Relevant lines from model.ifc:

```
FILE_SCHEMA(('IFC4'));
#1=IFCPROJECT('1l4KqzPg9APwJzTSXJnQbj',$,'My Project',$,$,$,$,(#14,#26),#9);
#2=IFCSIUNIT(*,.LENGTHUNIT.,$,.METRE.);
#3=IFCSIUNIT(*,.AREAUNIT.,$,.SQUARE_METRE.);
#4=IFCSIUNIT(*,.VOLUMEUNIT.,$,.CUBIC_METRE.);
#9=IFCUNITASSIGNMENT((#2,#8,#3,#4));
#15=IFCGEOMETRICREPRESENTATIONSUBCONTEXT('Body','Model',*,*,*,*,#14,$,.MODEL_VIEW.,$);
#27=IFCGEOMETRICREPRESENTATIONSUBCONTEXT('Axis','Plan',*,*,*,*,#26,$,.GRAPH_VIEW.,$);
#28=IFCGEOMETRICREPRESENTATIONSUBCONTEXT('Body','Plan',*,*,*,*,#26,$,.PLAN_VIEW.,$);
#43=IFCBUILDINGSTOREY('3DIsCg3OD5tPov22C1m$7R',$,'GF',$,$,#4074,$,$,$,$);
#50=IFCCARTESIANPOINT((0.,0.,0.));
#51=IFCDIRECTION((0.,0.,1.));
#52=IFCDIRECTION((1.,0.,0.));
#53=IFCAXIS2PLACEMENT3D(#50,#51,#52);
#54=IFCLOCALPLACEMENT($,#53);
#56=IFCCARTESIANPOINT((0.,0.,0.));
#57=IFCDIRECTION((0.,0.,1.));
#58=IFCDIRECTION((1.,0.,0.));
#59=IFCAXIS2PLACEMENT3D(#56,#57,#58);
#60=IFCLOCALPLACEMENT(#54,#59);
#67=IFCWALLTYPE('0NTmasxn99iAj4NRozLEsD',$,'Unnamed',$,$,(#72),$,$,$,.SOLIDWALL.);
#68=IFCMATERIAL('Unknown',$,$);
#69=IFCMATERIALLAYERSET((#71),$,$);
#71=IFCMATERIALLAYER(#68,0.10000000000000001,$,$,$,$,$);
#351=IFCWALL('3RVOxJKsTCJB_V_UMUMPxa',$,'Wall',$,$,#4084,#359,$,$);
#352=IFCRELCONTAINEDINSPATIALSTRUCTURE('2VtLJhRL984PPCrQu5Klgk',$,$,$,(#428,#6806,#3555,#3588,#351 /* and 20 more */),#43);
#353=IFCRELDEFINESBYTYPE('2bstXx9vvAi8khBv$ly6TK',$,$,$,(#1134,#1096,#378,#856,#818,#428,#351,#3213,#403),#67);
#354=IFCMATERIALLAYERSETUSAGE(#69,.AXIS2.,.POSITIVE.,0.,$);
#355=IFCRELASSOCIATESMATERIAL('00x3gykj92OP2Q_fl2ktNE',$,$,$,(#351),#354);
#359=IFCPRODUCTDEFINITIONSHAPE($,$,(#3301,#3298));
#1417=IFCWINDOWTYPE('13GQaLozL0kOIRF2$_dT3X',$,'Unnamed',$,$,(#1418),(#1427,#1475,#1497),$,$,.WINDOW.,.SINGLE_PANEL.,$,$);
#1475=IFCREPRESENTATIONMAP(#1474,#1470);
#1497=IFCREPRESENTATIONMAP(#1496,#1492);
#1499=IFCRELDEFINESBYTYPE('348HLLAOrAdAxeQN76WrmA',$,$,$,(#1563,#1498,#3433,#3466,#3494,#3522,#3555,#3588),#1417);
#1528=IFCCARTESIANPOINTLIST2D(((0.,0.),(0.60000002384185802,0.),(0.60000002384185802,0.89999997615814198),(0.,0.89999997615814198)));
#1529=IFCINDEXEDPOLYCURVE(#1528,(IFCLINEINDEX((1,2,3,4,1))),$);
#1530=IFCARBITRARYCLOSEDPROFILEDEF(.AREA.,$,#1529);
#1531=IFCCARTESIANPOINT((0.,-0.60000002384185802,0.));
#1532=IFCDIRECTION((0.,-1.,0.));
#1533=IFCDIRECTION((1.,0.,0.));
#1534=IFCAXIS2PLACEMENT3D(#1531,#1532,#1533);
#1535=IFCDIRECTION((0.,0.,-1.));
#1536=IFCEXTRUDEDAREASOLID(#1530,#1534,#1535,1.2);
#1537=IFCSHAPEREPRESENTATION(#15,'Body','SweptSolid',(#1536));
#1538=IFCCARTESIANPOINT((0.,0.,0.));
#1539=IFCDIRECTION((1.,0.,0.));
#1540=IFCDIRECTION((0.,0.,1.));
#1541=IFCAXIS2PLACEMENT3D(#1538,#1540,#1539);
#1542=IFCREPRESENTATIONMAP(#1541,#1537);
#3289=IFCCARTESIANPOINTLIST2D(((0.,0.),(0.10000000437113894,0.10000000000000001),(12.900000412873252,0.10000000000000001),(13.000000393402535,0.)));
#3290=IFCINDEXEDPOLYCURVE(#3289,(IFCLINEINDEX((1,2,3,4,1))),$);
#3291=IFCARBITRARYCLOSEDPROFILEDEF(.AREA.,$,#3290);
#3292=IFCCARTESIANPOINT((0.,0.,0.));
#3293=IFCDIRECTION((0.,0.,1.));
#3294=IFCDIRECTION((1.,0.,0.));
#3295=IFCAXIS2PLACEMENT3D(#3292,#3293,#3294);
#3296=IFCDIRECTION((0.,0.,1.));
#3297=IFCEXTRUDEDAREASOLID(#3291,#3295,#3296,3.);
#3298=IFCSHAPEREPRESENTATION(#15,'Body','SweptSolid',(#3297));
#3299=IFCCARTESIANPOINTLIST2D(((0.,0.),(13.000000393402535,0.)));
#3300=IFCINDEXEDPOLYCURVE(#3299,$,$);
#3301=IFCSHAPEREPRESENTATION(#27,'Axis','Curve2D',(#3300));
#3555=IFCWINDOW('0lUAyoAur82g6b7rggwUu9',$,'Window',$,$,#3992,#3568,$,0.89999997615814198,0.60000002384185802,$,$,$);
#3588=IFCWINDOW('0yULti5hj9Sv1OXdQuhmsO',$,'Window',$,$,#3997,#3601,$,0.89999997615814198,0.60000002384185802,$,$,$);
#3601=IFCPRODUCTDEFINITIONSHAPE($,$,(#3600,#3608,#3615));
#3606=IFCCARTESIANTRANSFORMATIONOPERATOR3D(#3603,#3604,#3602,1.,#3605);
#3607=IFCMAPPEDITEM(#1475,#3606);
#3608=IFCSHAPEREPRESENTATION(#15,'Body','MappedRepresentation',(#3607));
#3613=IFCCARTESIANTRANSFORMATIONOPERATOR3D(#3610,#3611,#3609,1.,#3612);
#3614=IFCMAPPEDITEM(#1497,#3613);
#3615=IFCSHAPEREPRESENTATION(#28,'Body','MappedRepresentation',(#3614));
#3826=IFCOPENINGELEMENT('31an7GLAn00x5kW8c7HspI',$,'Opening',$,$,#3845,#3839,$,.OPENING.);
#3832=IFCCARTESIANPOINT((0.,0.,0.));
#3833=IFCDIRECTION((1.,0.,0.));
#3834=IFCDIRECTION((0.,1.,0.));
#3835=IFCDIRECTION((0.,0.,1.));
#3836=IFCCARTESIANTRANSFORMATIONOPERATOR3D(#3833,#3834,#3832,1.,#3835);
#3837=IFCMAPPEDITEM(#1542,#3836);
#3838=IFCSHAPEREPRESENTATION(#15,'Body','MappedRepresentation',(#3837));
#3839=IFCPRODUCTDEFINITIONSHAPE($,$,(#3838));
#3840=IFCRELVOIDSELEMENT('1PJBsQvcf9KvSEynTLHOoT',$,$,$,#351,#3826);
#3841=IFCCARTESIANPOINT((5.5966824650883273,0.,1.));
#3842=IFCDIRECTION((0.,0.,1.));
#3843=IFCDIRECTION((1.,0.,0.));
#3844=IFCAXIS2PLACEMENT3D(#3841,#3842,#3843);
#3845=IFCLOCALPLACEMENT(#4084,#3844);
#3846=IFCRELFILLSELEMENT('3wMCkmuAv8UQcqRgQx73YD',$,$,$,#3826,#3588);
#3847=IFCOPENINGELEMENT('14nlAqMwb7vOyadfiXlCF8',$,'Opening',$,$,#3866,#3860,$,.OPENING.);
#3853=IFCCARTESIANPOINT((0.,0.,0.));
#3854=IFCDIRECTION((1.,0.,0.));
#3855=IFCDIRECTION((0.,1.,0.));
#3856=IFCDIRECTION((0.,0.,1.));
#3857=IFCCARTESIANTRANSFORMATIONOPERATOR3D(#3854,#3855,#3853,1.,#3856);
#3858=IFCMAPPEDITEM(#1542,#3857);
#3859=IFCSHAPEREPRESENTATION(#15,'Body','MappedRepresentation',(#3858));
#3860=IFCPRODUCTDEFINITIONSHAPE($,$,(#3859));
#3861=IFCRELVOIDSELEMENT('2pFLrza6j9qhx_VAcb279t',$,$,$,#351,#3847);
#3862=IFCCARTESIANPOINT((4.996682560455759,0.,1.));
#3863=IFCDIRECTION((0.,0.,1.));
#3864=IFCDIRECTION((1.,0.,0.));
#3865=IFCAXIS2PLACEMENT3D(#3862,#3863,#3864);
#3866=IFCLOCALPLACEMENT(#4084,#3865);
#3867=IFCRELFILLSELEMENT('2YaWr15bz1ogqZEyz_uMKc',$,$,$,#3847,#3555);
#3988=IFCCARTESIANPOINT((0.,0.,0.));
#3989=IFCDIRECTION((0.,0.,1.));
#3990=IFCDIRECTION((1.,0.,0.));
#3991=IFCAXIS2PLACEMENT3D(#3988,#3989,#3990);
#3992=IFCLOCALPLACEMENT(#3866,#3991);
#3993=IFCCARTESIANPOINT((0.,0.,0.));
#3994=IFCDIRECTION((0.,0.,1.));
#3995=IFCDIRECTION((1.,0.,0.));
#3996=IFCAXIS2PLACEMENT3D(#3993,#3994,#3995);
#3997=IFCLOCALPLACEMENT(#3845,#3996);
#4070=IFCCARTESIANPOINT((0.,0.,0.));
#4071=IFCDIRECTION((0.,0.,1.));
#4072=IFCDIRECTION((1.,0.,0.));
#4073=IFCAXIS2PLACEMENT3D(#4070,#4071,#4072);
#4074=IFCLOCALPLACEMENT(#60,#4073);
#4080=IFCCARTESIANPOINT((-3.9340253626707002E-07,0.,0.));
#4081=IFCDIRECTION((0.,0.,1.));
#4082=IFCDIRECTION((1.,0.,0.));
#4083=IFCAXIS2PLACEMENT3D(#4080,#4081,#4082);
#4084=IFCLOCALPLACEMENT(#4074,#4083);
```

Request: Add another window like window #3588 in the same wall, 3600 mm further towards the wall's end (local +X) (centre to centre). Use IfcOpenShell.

```python
import ifcopenshell
import ifcopenshell.api.feature
import ifcopenshell.api.geometry
import ifcopenshell.api.root
import ifcopenshell.geom
import ifcopenshell.util.element
import ifcopenshell.util.placement
import ifcopenshell.util.shape
import ifcopenshell.util.unit

model = ifcopenshell.open("model.ifc")
unit_scale = ifcopenshell.util.unit.calculate_unit_scale(model)
settings = ifcopenshell.geom.settings()


def volume(element):
    """Net volume in cubic metres, openings subtracted."""
    shape = ifcopenshell.geom.create_shape(settings, element)
    return ifcopenshell.util.shape.get_volume(shape.geometry)


window = model.by_guid("0yULti5hj9Sv1OXdQuhmsO")
opening = window.FillsVoids[0].RelatingOpeningElement
wall = opening.VoidsElements[0].RelatingBuildingElement
before = volume(wall)
shift = ifcopenshell.util.placement.get_local_placement(wall.ObjectPlacement)[:3, 0] * 3.6 / unit_scale

# copy_class copies the void relationship, type, container and properties, but no geometry.
new_opening = ifcopenshell.api.root.copy_class(model, product=opening)
new_opening.Representation = ifcopenshell.util.element.copy_deep(
    model, opening.Representation, exclude=["IfcGeometricRepresentationContext", "IfcRepresentationMap"]
)
new_window = ifcopenshell.api.root.copy_class(model, product=window)
new_window.Representation = ifcopenshell.util.element.copy_deep(
    model, window.Representation, exclude=["IfcGeometricRepresentationContext", "IfcRepresentationMap"]
)
ifcopenshell.api.feature.add_filling(model, opening=new_opening, element=new_window)

for old, new in ((opening, new_opening), (window, new_window)):
    matrix = ifcopenshell.util.placement.get_local_placement(old.ObjectPlacement)
    matrix[:3, 3] += shift
    ifcopenshell.api.geometry.edit_object_placement(model, product=new, matrix=matrix, is_si=False)

after = volume(wall)

print(f"wall volume {before:.3f} -> {after:.3f} m3")

model.write("model_v2.ifc")
```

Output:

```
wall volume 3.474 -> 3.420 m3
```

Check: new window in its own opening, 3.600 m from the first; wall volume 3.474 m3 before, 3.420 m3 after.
